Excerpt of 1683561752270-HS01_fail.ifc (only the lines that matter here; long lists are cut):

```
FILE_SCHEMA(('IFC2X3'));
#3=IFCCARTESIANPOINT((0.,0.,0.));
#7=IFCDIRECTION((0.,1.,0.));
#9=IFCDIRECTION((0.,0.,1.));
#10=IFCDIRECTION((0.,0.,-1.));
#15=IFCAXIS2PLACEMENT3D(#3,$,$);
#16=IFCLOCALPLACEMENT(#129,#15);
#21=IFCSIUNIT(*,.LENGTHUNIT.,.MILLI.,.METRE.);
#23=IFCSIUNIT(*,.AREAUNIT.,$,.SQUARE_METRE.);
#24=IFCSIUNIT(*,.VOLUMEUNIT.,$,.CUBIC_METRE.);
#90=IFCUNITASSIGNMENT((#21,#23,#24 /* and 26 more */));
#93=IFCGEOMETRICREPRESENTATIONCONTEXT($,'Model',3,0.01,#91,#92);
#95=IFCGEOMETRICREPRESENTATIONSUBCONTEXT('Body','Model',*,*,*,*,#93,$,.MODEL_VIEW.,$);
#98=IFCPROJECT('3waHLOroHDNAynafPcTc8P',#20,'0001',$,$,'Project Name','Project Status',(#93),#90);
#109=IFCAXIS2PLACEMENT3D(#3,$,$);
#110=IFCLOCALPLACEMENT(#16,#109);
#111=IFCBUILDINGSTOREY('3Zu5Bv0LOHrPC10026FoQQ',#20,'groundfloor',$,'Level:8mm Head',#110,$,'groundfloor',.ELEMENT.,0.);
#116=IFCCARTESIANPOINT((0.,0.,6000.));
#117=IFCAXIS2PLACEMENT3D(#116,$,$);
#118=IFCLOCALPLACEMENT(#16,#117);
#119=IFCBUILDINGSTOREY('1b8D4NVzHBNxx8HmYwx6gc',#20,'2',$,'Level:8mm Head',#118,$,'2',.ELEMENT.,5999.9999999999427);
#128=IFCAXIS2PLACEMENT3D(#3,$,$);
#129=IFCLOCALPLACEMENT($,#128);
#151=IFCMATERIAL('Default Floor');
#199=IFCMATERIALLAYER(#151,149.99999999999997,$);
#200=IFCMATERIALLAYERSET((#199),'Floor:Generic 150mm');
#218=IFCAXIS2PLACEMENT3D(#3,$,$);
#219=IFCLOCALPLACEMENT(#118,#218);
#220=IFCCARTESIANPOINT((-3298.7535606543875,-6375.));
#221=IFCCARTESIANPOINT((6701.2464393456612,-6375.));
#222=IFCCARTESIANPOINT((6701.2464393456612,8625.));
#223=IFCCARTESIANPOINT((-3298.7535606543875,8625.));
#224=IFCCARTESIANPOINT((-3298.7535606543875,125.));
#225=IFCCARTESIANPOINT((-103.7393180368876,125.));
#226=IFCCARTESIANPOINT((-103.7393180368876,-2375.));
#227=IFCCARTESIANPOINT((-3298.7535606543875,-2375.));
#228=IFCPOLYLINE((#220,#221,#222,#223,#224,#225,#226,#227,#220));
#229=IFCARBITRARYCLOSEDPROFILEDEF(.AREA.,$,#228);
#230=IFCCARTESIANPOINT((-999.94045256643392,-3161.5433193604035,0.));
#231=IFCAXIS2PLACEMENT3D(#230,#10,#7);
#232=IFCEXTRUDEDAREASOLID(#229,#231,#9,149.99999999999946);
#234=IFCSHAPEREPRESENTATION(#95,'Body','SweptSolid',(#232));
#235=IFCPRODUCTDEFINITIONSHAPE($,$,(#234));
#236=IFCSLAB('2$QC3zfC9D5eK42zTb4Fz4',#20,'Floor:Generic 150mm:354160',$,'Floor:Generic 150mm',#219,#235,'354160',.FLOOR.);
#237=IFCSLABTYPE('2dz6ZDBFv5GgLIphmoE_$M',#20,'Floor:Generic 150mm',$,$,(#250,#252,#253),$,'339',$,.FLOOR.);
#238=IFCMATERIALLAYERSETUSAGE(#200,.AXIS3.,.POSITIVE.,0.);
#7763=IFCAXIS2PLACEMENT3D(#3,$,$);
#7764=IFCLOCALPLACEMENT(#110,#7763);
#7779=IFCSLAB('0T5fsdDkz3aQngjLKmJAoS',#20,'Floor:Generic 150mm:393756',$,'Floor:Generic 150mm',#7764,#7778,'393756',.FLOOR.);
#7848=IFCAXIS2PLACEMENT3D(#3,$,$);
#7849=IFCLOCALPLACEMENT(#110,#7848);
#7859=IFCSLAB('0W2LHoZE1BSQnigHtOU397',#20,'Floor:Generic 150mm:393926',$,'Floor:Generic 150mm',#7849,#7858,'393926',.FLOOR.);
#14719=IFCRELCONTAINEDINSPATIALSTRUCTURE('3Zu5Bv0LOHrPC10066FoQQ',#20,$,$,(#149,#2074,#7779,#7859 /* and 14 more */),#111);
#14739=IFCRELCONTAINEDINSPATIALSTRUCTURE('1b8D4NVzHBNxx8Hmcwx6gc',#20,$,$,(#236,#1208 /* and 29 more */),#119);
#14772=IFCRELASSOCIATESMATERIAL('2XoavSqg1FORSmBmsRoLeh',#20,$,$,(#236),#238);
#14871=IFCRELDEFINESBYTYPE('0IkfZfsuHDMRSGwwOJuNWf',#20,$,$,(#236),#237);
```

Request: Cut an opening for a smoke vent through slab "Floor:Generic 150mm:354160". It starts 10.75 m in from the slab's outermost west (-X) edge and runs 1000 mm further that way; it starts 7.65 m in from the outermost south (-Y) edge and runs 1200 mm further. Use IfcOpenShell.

```python
import numpy as np
import ifcopenshell
import ifcopenshell.api.feature
import ifcopenshell.api.geometry
import ifcopenshell.api.root
import ifcopenshell.geom
import ifcopenshell.util.placement
import ifcopenshell.util.representation
import ifcopenshell.util.shape
import ifcopenshell.util.unit

model = ifcopenshell.open("1683561752270-HS01_fail.ifc")
unit_scale = ifcopenshell.util.unit.calculate_unit_scale(model)
settings = ifcopenshell.geom.settings()


def volume(element):
    """Net volume in cubic metres, openings subtracted."""
    shape = ifcopenshell.geom.create_shape(settings, element)
    return ifcopenshell.util.shape.get_volume(shape.geometry)


slab = model.by_id(236)
before = volume(slab)

# Extent in the slab's own axes, in metres. The edges named are its -X and -Y sides.
slab_shape = ifcopenshell.geom.create_shape(settings, slab)
vertices = ifcopenshell.util.shape.get_vertices(slab_shape.geometry)
x_min, y_min, bottom = vertices.min(axis=0)
top = vertices[:, 2].max()

opening = ifcopenshell.api.root.create_entity(model, ifc_class="IfcOpeningElement", name="Smoke vent opening")
context = ifcopenshell.util.representation.get_context(model, "Model", "Body", "MODEL_VIEW")
width, depth = 1, 1.2
outline = [(0.0, 0.0), (width, 0.0), (width, depth), (0.0, depth), (0.0, 0.0)]
# Overshoot both faces by 50 mm so the cut is clean.
shape = ifcopenshell.api.geometry.add_slab_representation(
    model, context=context, depth=top - bottom + 0.1, polyline=outline
)
ifcopenshell.api.geometry.assign_representation(model, product=opening, representation=shape)

matrix = ifcopenshell.util.placement.get_local_placement(slab.ObjectPlacement)
matrix[:, 3] = matrix @ np.append(np.array([x_min + 10.75, y_min + 7.65, bottom - 0.05]) / unit_scale, 1.0)
ifcopenshell.api.geometry.edit_object_placement(model, product=opening, matrix=matrix, is_si=False)
ifcopenshell.api.feature.add_feature(model, feature=opening, element=slab)

after = volume(slab)

print(f"slab volume {before:.3f} -> {after:.3f} m3")

model.write("1683561752270-HS01_fail-out.ifc")
```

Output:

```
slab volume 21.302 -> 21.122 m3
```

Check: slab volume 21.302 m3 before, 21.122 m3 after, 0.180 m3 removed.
